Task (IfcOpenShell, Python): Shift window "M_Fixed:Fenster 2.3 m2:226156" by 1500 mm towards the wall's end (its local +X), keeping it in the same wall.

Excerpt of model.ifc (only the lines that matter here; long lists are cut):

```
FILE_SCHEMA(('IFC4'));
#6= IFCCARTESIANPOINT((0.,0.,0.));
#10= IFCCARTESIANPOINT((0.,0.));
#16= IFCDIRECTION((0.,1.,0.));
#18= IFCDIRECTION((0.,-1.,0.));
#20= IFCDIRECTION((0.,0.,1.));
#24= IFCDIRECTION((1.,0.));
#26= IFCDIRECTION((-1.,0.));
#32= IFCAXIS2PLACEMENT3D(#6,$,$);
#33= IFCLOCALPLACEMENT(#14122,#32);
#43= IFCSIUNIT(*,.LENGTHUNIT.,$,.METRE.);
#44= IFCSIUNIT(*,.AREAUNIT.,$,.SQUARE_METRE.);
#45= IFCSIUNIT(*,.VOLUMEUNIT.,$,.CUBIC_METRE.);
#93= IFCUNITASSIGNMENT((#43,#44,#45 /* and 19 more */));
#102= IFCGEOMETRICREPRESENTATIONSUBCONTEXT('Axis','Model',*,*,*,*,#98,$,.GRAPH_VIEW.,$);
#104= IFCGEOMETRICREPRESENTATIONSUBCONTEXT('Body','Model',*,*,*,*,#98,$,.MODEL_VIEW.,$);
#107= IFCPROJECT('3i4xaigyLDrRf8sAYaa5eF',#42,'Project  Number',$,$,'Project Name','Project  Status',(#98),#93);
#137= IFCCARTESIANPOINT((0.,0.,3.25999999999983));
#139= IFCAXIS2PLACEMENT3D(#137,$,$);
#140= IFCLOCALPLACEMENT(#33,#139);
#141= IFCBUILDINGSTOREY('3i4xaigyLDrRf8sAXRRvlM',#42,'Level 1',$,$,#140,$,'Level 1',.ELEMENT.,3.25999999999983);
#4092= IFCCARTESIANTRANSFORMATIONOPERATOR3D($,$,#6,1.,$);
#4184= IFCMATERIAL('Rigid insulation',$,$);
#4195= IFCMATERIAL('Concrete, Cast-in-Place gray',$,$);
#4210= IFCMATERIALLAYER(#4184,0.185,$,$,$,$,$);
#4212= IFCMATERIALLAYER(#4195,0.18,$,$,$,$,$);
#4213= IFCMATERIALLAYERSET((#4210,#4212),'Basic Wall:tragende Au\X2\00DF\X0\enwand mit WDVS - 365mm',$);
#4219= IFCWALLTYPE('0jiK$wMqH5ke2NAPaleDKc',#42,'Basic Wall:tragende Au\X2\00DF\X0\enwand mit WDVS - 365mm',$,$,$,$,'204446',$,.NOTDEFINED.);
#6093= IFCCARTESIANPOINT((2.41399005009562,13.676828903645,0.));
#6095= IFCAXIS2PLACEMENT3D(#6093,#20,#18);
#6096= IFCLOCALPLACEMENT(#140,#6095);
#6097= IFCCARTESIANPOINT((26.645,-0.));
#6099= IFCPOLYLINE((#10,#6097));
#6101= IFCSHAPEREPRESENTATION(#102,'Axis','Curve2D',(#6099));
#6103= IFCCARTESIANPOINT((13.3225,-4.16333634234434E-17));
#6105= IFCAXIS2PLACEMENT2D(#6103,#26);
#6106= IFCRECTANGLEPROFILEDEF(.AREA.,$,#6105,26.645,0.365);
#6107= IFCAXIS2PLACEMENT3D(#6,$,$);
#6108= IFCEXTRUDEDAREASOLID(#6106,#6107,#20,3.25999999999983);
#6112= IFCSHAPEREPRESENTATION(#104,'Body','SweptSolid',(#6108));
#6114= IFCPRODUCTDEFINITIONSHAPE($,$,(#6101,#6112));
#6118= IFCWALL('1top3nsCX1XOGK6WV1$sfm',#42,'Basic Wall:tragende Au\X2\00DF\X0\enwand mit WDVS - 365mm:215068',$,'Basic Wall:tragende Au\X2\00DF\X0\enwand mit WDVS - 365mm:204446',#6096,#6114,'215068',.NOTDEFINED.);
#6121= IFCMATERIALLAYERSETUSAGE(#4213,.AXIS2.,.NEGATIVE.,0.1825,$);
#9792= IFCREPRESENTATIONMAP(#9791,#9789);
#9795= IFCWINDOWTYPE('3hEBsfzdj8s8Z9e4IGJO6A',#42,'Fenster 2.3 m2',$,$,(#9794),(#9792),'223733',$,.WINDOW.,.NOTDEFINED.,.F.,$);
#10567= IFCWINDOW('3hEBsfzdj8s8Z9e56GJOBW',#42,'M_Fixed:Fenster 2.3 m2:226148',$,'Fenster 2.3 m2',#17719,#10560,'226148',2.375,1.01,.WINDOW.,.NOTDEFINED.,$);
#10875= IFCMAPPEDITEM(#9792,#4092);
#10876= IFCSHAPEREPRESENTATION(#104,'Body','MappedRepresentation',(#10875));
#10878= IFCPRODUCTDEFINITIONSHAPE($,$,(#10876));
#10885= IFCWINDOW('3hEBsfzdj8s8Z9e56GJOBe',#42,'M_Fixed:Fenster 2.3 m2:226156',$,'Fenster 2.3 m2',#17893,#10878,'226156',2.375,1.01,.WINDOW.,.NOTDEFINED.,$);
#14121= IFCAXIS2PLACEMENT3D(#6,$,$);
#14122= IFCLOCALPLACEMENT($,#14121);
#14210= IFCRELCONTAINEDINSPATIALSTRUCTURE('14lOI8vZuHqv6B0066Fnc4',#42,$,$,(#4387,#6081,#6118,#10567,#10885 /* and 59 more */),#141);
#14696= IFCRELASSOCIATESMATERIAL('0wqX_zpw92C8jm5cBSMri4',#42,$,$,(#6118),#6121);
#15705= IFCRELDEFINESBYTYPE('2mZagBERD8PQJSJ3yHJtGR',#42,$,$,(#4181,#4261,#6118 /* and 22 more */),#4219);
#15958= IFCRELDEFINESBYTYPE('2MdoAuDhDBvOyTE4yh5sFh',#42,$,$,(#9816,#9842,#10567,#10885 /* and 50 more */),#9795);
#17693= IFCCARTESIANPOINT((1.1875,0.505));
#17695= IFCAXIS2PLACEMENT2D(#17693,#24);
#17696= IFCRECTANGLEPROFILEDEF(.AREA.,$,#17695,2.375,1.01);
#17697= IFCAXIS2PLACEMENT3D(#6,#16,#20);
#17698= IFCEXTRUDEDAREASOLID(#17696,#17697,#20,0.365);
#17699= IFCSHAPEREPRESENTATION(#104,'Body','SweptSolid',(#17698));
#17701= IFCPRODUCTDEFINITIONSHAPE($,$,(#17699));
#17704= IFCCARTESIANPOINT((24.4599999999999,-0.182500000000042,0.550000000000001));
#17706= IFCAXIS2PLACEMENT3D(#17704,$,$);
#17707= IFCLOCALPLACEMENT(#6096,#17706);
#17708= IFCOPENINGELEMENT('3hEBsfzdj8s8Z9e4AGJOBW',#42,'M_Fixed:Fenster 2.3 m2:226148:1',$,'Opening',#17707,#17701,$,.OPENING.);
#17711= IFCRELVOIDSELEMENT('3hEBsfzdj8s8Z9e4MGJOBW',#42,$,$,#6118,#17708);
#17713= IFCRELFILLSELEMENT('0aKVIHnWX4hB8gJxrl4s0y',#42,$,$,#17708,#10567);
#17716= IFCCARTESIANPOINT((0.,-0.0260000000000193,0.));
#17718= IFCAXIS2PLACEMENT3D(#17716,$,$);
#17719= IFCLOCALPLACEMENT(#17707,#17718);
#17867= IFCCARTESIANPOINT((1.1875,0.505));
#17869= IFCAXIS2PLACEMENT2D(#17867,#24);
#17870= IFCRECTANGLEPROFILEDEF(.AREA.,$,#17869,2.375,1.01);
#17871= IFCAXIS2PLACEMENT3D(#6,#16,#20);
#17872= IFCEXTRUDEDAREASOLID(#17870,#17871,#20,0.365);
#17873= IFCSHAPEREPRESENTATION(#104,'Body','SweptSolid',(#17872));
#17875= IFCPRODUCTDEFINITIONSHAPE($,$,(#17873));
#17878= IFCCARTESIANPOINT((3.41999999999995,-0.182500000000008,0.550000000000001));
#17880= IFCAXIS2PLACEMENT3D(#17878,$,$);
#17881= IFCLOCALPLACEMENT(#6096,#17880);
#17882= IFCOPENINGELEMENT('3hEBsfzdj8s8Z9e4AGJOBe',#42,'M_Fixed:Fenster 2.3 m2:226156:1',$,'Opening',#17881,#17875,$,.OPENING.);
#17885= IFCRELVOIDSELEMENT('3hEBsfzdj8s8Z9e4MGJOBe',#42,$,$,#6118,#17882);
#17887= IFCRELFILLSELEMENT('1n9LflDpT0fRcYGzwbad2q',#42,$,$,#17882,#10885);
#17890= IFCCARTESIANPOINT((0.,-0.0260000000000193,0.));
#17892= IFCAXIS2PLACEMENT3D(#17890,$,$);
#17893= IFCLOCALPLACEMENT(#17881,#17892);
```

```python
import ifcopenshell
import ifcopenshell.api.geometry
import ifcopenshell.util.placement

model = ifcopenshell.open("model.ifc")

window = model.by_id(10885)
opening = window.FillsVoids[0].RelatingOpeningElement
wall = opening.VoidsElements[0].RelatingBuildingElement

wall_matrix = ifcopenshell.util.placement.get_local_placement(wall.ObjectPlacement)
shift = wall_matrix[:3, 0] * 1.5
before = ifcopenshell.util.placement.get_local_placement(window.ObjectPlacement)[:3, 3].copy()

# The window is placed relative to its opening, so it follows when the opening moves.
matrix = ifcopenshell.util.placement.get_local_placement(opening.ObjectPlacement)
matrix[:3, 3] += shift
ifcopenshell.api.geometry.edit_object_placement(
    model, product=opening, matrix=matrix, is_si=False, should_transform_children=True
)

after = ifcopenshell.util.placement.get_local_placement(window.ObjectPlacement)[:3, 3]
print("window moved by", (after - before).round(3) + 0.0)

model.write("model_edited.ifc")
```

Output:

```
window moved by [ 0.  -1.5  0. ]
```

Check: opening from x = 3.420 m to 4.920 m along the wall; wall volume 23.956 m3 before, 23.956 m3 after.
